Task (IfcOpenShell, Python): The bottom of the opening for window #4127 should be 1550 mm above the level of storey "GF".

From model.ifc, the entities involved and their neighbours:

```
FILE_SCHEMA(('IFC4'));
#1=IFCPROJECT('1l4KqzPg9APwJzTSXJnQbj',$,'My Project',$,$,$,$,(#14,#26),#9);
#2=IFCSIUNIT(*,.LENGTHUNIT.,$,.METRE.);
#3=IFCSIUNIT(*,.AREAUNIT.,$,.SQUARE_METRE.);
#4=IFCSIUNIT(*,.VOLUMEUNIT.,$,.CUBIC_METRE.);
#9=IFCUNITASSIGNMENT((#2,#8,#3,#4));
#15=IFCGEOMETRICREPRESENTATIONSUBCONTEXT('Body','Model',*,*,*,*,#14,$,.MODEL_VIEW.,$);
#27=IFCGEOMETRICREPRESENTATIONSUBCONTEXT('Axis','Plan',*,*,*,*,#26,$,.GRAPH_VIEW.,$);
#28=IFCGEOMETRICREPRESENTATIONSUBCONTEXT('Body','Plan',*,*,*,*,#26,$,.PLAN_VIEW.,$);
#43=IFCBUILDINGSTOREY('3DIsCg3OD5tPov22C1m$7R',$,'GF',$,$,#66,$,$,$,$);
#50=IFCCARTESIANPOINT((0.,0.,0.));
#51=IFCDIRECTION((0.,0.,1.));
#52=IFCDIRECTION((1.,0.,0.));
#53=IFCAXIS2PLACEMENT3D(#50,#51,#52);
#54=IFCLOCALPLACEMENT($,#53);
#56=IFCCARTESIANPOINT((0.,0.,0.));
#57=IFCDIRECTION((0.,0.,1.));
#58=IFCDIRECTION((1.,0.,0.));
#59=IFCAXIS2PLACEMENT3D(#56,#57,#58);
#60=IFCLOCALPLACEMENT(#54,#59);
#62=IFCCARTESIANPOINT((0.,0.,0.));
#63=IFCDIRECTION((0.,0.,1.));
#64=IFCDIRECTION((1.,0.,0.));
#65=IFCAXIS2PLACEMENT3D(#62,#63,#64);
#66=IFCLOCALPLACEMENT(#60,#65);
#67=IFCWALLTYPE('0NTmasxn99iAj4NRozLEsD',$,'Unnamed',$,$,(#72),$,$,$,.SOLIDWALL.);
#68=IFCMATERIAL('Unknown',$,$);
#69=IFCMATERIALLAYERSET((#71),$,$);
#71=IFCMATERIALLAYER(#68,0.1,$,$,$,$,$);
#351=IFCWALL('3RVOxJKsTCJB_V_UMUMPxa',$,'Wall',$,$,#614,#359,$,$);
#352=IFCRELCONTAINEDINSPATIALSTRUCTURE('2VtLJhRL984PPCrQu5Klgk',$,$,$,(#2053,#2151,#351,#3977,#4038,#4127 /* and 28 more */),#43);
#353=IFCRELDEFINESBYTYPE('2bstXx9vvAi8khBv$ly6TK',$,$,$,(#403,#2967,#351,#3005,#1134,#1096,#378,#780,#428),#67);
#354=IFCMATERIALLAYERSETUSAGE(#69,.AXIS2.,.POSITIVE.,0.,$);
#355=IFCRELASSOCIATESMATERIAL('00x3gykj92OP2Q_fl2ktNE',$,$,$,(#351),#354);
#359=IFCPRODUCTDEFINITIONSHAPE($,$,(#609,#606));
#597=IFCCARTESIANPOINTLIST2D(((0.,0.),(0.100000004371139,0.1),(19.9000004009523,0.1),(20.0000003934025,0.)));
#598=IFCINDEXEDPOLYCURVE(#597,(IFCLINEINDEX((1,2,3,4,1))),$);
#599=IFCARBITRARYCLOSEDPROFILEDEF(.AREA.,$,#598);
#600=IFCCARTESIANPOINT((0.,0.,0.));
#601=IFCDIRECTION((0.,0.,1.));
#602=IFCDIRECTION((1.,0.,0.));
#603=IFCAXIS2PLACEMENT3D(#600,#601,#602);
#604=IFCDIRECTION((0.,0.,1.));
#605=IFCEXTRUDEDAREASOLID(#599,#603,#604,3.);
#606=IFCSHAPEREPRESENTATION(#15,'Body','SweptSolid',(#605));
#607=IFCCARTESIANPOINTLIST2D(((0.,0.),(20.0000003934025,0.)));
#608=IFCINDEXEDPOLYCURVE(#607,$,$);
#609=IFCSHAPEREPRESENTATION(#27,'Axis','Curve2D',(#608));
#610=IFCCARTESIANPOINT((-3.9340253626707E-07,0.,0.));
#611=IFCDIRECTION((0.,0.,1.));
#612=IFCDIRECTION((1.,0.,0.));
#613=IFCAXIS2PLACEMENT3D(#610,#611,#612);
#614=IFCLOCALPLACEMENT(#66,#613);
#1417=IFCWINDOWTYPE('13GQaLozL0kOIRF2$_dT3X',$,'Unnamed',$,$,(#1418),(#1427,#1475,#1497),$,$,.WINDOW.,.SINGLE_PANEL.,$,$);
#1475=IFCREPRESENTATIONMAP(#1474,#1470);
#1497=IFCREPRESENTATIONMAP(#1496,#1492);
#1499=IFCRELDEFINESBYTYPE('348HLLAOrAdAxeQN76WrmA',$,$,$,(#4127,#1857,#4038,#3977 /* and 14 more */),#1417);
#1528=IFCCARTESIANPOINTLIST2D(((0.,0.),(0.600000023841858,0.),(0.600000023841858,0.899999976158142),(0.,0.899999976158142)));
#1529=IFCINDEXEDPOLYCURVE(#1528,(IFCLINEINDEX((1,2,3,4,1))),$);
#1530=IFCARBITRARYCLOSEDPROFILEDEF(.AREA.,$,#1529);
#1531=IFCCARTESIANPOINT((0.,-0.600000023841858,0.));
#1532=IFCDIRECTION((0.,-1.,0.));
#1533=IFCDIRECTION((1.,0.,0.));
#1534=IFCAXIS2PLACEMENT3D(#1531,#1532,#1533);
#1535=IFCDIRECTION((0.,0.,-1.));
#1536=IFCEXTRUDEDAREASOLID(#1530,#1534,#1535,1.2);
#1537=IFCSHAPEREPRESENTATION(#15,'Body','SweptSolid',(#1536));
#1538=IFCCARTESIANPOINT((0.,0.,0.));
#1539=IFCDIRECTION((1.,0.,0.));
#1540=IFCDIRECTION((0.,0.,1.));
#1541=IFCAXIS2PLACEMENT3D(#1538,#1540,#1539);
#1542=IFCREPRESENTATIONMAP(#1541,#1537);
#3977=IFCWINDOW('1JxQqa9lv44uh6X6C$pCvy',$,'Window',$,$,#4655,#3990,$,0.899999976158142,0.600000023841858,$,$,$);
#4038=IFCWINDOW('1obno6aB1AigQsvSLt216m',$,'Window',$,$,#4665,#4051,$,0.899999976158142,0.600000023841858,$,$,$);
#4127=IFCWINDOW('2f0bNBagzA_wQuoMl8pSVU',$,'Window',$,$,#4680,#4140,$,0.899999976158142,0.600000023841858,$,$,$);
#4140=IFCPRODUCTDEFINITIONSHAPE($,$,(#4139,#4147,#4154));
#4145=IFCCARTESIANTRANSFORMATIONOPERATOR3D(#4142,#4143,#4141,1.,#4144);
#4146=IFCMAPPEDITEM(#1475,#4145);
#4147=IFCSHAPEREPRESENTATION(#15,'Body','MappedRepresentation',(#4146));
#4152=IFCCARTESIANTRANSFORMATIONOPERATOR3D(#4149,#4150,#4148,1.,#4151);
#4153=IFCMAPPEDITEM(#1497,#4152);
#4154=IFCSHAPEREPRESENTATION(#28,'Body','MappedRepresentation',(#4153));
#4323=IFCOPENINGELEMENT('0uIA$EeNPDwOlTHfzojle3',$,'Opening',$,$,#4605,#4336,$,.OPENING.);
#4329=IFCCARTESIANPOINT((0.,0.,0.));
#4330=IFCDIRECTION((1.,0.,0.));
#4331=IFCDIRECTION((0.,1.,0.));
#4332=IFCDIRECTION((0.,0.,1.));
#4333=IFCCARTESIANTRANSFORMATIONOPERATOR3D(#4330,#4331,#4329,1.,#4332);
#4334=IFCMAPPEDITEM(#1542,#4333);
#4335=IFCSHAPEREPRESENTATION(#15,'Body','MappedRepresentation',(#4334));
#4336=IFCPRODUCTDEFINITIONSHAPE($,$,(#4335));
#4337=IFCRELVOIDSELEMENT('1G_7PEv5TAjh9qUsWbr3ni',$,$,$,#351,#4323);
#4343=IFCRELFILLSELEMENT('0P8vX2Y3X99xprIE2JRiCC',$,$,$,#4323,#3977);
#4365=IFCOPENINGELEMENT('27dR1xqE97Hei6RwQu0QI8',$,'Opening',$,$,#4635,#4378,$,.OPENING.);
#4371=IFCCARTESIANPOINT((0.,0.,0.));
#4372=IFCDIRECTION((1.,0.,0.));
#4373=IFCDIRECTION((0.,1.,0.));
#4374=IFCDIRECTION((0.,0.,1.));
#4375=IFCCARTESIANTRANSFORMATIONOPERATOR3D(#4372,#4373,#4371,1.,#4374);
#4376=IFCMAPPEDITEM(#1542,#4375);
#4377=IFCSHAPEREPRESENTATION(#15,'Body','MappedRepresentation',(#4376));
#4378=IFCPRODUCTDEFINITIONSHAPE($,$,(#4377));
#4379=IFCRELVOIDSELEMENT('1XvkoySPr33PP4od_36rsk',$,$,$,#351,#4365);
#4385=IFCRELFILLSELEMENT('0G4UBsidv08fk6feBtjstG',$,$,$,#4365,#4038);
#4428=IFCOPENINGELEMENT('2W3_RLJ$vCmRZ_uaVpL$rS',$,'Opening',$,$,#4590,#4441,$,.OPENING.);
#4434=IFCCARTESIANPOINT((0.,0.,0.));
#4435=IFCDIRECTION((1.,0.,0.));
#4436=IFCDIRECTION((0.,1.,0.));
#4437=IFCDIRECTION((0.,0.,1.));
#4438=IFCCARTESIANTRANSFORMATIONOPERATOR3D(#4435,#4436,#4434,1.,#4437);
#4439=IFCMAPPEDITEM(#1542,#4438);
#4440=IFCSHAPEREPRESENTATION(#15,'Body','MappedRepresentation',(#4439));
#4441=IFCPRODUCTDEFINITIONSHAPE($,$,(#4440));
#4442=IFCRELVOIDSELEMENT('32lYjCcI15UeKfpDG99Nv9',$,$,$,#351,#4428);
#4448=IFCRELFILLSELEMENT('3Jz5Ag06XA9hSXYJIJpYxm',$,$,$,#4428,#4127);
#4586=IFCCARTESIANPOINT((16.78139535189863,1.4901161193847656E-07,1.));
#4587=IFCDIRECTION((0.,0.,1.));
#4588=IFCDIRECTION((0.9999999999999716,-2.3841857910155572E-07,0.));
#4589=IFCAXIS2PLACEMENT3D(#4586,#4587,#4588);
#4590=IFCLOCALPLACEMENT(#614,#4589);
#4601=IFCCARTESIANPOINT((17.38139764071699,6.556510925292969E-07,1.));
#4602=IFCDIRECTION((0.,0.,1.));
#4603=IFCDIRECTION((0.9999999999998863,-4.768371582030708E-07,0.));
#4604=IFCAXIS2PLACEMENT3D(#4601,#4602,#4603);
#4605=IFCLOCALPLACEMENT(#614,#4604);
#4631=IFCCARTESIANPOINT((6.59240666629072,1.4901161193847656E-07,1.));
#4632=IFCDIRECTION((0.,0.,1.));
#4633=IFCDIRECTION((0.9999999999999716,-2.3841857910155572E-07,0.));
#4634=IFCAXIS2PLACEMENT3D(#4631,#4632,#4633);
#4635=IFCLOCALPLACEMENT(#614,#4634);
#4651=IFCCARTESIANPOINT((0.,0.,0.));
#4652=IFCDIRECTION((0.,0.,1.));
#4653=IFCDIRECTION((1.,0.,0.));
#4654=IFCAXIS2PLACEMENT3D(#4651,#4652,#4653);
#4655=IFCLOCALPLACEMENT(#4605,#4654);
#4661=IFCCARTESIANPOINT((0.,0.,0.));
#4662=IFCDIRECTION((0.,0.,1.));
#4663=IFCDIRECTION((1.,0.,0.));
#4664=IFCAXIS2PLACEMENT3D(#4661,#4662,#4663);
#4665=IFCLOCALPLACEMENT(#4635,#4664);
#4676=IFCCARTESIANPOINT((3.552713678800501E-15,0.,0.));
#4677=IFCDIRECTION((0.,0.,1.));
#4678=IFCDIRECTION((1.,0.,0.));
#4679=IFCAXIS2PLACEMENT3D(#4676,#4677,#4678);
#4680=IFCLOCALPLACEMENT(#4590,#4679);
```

```python
import numpy as np
import ifcopenshell
import ifcopenshell.api.geometry
import ifcopenshell.geom
import ifcopenshell.util.element
import ifcopenshell.util.placement
import ifcopenshell.util.shape
import ifcopenshell.util.unit

model = ifcopenshell.open("model.ifc")
unit_scale = ifcopenshell.util.unit.calculate_unit_scale(model)

window = model.by_guid("2f0bNBagzA_wQuoMl8pSVU")
opening = window.FillsVoids[0].RelatingOpeningElement
storey = ifcopenshell.util.element.get_container(window, ifc_class="IfcBuildingStorey")
level = ifcopenshell.util.placement.get_local_placement(storey.ObjectPlacement)[2, 3]

# The opening's origin need not be at the sill, so measure its lowest point.
shape = ifcopenshell.geom.create_shape(ifcopenshell.geom.settings(), opening)
bottom = ifcopenshell.util.shape.get_shape_bottom_elevation(shape, shape.geometry) / unit_scale
dz = level + 1.55 / unit_scale - bottom

shift = np.array([0.0, 0.0, dz])
# The window is placed relative to its opening, so it follows when the opening moves.
matrix = ifcopenshell.util.placement.get_local_placement(opening.ObjectPlacement)
matrix[:3, 3] += shift
ifcopenshell.api.geometry.edit_object_placement(
    model, product=opening, matrix=matrix, is_si=False, should_transform_children=True
)

print(f"moved by {dz * unit_scale:+.3f} m")

model.write("model_updated.ifc")
```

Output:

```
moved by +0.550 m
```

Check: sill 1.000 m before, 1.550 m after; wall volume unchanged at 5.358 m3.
